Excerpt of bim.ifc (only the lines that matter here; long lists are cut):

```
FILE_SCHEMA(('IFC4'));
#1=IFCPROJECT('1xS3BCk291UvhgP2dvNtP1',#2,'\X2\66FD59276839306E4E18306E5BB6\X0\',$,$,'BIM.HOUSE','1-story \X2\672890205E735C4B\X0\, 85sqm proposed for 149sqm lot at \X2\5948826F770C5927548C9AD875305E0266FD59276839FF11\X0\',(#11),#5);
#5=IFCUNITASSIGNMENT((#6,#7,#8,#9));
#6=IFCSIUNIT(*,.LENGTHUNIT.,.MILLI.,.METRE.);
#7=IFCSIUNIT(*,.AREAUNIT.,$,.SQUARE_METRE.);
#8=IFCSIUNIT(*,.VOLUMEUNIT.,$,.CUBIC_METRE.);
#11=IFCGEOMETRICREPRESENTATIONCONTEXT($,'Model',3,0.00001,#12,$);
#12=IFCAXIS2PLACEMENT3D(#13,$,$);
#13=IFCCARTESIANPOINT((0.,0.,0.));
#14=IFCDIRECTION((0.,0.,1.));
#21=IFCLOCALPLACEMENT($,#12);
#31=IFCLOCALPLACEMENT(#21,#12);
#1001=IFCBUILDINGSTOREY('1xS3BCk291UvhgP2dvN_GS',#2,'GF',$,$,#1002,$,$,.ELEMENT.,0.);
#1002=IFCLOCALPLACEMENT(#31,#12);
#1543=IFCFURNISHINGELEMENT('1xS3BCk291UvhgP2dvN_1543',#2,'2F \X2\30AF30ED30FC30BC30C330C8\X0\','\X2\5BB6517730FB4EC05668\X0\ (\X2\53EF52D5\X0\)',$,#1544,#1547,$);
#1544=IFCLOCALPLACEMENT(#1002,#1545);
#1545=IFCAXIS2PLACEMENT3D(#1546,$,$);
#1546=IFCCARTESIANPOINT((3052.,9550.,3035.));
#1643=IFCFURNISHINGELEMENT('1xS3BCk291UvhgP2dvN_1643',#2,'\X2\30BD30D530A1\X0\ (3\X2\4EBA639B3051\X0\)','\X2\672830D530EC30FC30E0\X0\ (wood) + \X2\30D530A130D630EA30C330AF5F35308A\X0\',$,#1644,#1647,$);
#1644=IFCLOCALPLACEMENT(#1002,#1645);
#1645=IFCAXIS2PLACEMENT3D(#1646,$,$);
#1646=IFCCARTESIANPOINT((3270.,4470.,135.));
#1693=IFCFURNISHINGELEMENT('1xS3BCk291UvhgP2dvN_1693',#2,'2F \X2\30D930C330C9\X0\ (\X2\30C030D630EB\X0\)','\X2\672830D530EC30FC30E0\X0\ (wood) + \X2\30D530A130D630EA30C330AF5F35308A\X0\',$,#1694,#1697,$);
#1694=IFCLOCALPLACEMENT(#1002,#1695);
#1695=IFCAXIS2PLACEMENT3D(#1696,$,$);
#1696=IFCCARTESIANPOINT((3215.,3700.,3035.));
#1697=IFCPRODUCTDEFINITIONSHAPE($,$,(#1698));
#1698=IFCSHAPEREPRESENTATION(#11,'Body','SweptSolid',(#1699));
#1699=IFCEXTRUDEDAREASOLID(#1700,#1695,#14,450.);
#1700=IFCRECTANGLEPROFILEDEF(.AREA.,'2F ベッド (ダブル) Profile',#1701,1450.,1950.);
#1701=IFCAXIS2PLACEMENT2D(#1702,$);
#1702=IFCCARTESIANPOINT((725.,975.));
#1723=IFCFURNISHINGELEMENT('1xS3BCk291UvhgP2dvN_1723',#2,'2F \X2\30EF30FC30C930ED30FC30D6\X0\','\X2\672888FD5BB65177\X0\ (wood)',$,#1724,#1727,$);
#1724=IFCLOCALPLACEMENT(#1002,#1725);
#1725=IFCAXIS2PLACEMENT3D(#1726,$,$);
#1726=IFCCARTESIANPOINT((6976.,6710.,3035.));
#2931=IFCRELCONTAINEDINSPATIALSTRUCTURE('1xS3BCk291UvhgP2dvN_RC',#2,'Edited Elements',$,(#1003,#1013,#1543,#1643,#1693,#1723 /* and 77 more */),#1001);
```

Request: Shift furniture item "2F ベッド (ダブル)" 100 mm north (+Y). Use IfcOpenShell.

```python
import ifcopenshell
import ifcopenshell.api.geometry
import ifcopenshell.util.placement

model = ifcopenshell.open("bim.ifc")

item = model.by_id(1693)
matrix = ifcopenshell.util.placement.get_local_placement(item.ObjectPlacement)
matrix[1, 3] += 100.0
ifcopenshell.api.geometry.edit_object_placement(model, product=item, matrix=matrix, is_si=False)

print(ifcopenshell.util.placement.get_local_placement(item.ObjectPlacement).round(3) + 0.0)

model.write("bim_edited.ifc")
```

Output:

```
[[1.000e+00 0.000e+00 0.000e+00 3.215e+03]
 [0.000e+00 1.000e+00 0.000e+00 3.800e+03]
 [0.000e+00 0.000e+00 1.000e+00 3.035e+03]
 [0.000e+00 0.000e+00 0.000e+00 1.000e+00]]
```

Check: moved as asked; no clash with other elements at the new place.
